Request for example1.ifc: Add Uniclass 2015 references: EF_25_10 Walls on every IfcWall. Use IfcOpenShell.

First a look at what the model holds.

```python
import ifcopenshell

model = ifcopenshell.open("example1.ifc")
print(model.schema)
print("classifications:", [c.Name for c in model.by_type("IfcClassification")])
for ifc_class in ("IfcDoor", "IfcRoof", "IfcStair", "IfcWall", "IfcWindow"):
    print(ifc_class, len(model.by_type(ifc_class)))
```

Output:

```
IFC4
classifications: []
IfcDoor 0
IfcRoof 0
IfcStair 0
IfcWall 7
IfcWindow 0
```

```python
import ifcopenshell
import ifcopenshell.api.classification

model = ifcopenshell.open("example1.ifc")

system = ifcopenshell.api.classification.add_classification(model, classification="Uniclass 2015")

codes = {
    "IfcWall": ("EF_25_10", "Walls"),
}
for ifc_class, (code, name) in codes.items():
    products = model.by_type(ifc_class)
    ifcopenshell.api.classification.add_reference(
        model, products=products, classification=system, identification=code, name=name
    )
    print(code, len(products))

model.write("example1_v2.ifc")
```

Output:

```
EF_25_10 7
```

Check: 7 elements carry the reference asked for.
